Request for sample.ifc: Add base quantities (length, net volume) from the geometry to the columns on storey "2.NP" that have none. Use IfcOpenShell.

First a look at what the model holds.

```python
import ifcopenshell
import ifcopenshell.util.element
import ifcopenshell.util.unit

model = ifcopenshell.open("sample.ifc")
print(model.schema)
for unit_type in ("LENGTHUNIT", "AREAUNIT", "VOLUMEUNIT"):
    print(unit_type, ifcopenshell.util.unit.calculate_unit_scale(model, unit_type))
storey = next(s for s in model.by_type("IfcBuildingStorey") if s.Name == "2.NP")
columns = [e for e in ifcopenshell.util.element.get_decomposition(storey) if e.is_a("IfcColumn")]
for e in sorted(columns, key=lambda e: e.id()):
    print(e.id(), e.is_a(), e.Name, list(ifcopenshell.util.element.get_psets(e, qtos_only=True)), sep=" | ")
```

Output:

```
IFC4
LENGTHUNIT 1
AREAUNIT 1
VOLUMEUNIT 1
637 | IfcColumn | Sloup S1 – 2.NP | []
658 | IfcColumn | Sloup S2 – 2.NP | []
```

```python
import ifcopenshell
import ifcopenshell.api.pset
import ifcopenshell.geom
import ifcopenshell.util.element
import ifcopenshell.util.shape
import ifcopenshell.util.unit

model = ifcopenshell.open("sample.ifc")
unit_scale = ifcopenshell.util.unit.calculate_unit_scale(model)
volume_scale = ifcopenshell.util.unit.calculate_unit_scale(model, "VOLUMEUNIT")
settings = ifcopenshell.geom.settings()

storey = next(s for s in model.by_type("IfcBuildingStorey") if s.Name == "2.NP")
columns = [e for e in ifcopenshell.util.element.get_decomposition(storey) if e.is_a("IfcColumn")]

for e in sorted(columns, key=lambda e: e.id()):
    if ifcopenshell.util.element.get_psets(e, qtos_only=True, should_inherit=False):
        continue
    # Geometry comes back in metres, in the element's own axes.
    shape = ifcopenshell.geom.create_shape(settings, e)
    values = {
        "Length": ifcopenshell.util.shape.get_z(shape.geometry) / unit_scale,
        "NetVolume": ifcopenshell.util.shape.get_volume(shape.geometry) / volume_scale,
    }
    qto = ifcopenshell.api.pset.add_qto(model, product=e, name="Qto_ColumnBaseQuantities")
    ifcopenshell.api.pset.edit_qto(model, qto=qto, properties=values)
    print(e.id(), {k: round(v, 3) for k, v in values.items()})

model.write("sample_v2.ifc")
```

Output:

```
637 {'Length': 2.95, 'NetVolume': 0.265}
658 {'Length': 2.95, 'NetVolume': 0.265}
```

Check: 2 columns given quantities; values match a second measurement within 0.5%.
